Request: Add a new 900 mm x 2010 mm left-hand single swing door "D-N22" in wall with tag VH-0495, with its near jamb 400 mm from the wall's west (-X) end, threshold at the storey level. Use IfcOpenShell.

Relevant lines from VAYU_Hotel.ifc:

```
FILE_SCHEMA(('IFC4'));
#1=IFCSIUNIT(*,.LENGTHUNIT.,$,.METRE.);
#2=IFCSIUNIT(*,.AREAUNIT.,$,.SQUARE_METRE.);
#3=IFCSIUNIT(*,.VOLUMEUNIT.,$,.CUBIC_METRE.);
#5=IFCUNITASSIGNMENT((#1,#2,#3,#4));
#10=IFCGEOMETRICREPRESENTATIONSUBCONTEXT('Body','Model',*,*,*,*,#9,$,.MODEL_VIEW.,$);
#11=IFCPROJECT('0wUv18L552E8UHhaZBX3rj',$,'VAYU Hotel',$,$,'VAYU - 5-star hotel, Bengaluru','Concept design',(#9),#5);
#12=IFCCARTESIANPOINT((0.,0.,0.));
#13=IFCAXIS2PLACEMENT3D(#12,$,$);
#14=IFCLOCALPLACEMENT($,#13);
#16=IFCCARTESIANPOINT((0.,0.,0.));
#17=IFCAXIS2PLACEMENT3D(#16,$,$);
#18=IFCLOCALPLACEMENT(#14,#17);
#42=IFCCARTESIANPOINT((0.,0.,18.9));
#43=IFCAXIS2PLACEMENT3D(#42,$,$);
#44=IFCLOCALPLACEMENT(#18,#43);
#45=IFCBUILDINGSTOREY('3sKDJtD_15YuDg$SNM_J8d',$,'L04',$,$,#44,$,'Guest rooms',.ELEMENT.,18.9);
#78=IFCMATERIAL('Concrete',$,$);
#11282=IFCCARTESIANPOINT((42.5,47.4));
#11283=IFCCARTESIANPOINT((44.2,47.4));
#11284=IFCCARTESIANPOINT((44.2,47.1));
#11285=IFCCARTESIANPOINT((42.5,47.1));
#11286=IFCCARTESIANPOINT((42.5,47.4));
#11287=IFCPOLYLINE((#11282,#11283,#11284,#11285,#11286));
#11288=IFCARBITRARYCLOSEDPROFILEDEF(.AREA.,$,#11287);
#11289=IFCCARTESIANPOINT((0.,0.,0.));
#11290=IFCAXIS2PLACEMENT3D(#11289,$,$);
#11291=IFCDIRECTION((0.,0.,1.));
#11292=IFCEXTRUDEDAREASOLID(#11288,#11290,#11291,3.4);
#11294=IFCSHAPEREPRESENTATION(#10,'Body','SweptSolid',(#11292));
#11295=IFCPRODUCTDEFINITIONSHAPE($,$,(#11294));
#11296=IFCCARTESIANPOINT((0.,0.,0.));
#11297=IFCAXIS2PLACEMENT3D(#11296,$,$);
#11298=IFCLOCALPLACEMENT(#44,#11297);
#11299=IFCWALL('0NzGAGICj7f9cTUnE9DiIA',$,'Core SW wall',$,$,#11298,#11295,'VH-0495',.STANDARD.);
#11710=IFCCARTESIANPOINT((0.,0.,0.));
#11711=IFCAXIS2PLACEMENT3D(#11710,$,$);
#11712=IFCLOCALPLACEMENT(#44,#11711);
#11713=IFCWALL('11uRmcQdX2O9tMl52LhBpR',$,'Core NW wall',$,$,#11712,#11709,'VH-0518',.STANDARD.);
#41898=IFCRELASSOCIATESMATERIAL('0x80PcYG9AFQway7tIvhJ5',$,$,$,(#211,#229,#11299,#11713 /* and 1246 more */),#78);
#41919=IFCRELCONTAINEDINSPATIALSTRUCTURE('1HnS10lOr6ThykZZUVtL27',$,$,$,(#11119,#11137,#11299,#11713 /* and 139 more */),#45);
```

```python
import numpy as np
import ifcopenshell
import ifcopenshell.api.feature
import ifcopenshell.api.geometry
import ifcopenshell.api.root
import ifcopenshell.api.spatial
import ifcopenshell.geom
import ifcopenshell.util.element
import ifcopenshell.util.placement
import ifcopenshell.util.representation
import ifcopenshell.util.shape
import ifcopenshell.util.unit

model = ifcopenshell.open("VAYU_Hotel.ifc")
unit_scale = ifcopenshell.util.unit.calculate_unit_scale(model)
settings = ifcopenshell.geom.settings()


def volume(element):
    """Net volume in cubic metres, openings subtracted."""
    shape = ifcopenshell.geom.create_shape(settings, element)
    return ifcopenshell.util.shape.get_volume(shape.geometry)


wall = model.by_guid("0NzGAGICj7f9cTUnE9DiIA")
storey = ifcopenshell.util.element.get_container(wall, ifc_class="IfcBuildingStorey")
context = ifcopenshell.util.representation.get_context(model, "Model", "Body", "MODEL_VIEW")
before = volume(wall)

width, height, from_end, sill = 0.9, 2.01, 0.4, 0.0  # metres

# The wall runs along its own X axis, and the end named is its -X end.
wall_shape = ifcopenshell.geom.create_shape(settings, wall)
x, y, z = ifcopenshell.util.shape.get_vertices(wall_shape.geometry).T
start = x.min() + from_end
face, thickness = float(y.min()), float(y.max() - y.min())
wall_matrix = ifcopenshell.util.placement.get_local_placement(wall.ObjectPlacement)
level = ifcopenshell.util.placement.get_local_placement(storey.ObjectPlacement)[2, 3]


def in_wall(x, y):
    """Placement at x, y metres in the wall's axes, at sill height."""
    matrix = wall_matrix.copy()
    matrix[:, 3] = wall_matrix @ np.array([x / unit_scale, y / unit_scale, 0.0, 1.0])
    matrix[2, 3] = level + sill / unit_scale
    return matrix


# Opening: a box that overshoots both wall faces by 50 mm.
opening = ifcopenshell.api.root.create_entity(model, ifc_class="IfcOpeningElement", predefined_type="OPENING")
box = ifcopenshell.api.geometry.add_wall_representation(
    model, context=context, length=width, height=height, thickness=thickness + 0.1
)
ifcopenshell.api.geometry.assign_representation(model, product=opening, representation=box)
ifcopenshell.api.geometry.edit_object_placement(model, product=opening, matrix=in_wall(start, face - 0.05), is_si=False)
ifcopenshell.api.feature.add_feature(model, feature=opening, element=wall)

door = ifcopenshell.api.root.create_entity(model, ifc_class="IfcDoor", name="D-N22", predefined_type="DOOR")
door.OverallWidth, door.OverallHeight = width / unit_scale, height / unit_scale
door.OperationType = "SINGLE_SWING_LEFT"
body = ifcopenshell.api.geometry.add_door_representation(
    model,
    context=context,
    overall_width=door.OverallWidth,
    overall_height=door.OverallHeight,
    operation_type="SINGLE_SWING_LEFT",
    lining_properties={"LiningDepth": thickness / unit_scale, "ThresholdDepth": thickness / unit_scale},
)
ifcopenshell.api.geometry.assign_representation(model, product=door, representation=body)
ifcopenshell.api.spatial.assign_container(model, products=[door], relating_structure=storey)
ifcopenshell.api.feature.add_filling(model, opening=opening, element=door)

# The lining spans the wall, so the door starts at the wall face.
ifcopenshell.api.geometry.edit_object_placement(model, product=door, matrix=in_wall(start, face), is_si=False)

after = volume(wall)

print(f"wall volume {before:.3f} -> {after:.3f} m3")

model.write("VAYU_Hotel_edited.ifc")
```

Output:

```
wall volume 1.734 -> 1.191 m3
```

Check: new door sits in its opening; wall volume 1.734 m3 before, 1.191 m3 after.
